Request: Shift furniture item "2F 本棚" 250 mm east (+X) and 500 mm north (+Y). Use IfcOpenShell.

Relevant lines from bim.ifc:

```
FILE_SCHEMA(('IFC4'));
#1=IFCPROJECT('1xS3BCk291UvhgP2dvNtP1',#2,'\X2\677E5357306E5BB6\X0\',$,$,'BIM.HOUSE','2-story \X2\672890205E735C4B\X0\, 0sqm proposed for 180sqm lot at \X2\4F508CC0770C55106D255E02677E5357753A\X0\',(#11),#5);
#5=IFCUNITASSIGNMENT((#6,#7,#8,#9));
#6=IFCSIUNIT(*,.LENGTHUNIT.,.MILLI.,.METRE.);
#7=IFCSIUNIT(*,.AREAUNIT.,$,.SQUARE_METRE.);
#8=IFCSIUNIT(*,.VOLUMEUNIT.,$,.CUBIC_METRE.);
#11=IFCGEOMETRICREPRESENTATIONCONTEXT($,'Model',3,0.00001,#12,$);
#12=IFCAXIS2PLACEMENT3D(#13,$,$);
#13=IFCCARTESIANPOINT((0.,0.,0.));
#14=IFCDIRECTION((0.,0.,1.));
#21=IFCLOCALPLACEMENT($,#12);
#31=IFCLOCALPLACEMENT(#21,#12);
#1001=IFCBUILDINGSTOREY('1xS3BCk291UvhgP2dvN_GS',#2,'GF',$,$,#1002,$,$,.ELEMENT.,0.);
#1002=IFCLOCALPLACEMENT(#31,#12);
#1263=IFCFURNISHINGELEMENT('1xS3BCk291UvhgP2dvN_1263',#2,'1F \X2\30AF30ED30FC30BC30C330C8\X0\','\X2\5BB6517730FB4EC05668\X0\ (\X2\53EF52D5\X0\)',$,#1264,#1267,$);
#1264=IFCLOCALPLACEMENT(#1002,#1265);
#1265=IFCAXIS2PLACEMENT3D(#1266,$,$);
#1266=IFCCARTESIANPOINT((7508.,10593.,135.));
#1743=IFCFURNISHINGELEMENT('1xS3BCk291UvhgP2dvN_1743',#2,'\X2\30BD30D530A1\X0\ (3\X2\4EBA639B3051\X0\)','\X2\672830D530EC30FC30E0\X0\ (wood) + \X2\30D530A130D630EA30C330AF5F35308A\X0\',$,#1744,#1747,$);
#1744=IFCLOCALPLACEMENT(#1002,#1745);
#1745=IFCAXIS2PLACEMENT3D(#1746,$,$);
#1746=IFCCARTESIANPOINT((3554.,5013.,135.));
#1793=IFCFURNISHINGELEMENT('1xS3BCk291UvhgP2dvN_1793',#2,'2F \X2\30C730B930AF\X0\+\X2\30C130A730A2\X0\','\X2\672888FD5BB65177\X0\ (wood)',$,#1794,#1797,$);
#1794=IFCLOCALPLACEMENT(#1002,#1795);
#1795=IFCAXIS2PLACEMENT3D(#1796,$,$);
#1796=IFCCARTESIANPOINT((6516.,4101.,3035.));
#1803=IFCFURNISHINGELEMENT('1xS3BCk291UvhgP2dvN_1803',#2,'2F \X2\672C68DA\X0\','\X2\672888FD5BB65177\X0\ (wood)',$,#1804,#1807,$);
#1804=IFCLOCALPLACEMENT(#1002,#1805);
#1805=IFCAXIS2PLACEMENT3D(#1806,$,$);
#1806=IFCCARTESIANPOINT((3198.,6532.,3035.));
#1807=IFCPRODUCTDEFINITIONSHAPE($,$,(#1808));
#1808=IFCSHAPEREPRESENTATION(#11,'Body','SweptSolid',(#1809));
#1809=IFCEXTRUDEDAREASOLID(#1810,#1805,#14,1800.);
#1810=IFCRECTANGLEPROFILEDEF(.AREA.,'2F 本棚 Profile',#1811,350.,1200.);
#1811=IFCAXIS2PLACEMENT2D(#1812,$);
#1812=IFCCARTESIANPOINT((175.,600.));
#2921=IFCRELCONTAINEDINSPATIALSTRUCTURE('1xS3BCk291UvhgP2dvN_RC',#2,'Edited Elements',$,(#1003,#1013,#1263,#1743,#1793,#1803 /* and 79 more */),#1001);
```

```python
import ifcopenshell
import ifcopenshell.api.geometry
import ifcopenshell.util.placement
import ifcopenshell.util.unit

model = ifcopenshell.open("bim.ifc")
unit_scale = ifcopenshell.util.unit.calculate_unit_scale(model)

item = model.by_guid("1xS3BCk291UvhgP2dvN_1803")
matrix = ifcopenshell.util.placement.get_local_placement(item.ObjectPlacement)
matrix[0, 3] += 0.25 / unit_scale
matrix[1, 3] += 0.5 / unit_scale
ifcopenshell.api.geometry.edit_object_placement(model, product=item, matrix=matrix, is_si=False)

print(ifcopenshell.util.placement.get_local_placement(item.ObjectPlacement).round(3) + 0.0)

model.write("bim-out.ifc")
```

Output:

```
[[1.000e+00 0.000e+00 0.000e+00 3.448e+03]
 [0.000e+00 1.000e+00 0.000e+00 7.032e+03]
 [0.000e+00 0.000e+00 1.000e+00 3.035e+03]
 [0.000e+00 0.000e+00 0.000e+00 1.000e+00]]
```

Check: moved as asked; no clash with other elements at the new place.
